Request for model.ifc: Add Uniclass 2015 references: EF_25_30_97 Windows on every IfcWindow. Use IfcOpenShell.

First a look at what the model holds.

```python
import ifcopenshell

model = ifcopenshell.open("model.ifc")
print(model.schema)
print("classifications:", [c.Name for c in model.by_type("IfcClassification")])
for ifc_class in ("IfcDoor", "IfcRoof", "IfcStair", "IfcWall", "IfcWindow"):
    print(ifc_class, len(model.by_type(ifc_class)))
```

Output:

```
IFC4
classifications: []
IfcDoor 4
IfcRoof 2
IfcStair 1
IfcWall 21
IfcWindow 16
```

```python
import ifcopenshell
import ifcopenshell.api.classification

model = ifcopenshell.open("model.ifc")

system = ifcopenshell.api.classification.add_classification(model, classification="Uniclass 2015")

codes = {
    "IfcWindow": ("EF_25_30_97", "Windows"),
}
for ifc_class, (code, name) in codes.items():
    products = model.by_type(ifc_class)
    ifcopenshell.api.classification.add_reference(
        model, products=products, classification=system, identification=code, name=name
    )
    print(code, len(products))

model.write("model_updated.ifc")
```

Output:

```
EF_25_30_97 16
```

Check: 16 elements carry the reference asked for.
